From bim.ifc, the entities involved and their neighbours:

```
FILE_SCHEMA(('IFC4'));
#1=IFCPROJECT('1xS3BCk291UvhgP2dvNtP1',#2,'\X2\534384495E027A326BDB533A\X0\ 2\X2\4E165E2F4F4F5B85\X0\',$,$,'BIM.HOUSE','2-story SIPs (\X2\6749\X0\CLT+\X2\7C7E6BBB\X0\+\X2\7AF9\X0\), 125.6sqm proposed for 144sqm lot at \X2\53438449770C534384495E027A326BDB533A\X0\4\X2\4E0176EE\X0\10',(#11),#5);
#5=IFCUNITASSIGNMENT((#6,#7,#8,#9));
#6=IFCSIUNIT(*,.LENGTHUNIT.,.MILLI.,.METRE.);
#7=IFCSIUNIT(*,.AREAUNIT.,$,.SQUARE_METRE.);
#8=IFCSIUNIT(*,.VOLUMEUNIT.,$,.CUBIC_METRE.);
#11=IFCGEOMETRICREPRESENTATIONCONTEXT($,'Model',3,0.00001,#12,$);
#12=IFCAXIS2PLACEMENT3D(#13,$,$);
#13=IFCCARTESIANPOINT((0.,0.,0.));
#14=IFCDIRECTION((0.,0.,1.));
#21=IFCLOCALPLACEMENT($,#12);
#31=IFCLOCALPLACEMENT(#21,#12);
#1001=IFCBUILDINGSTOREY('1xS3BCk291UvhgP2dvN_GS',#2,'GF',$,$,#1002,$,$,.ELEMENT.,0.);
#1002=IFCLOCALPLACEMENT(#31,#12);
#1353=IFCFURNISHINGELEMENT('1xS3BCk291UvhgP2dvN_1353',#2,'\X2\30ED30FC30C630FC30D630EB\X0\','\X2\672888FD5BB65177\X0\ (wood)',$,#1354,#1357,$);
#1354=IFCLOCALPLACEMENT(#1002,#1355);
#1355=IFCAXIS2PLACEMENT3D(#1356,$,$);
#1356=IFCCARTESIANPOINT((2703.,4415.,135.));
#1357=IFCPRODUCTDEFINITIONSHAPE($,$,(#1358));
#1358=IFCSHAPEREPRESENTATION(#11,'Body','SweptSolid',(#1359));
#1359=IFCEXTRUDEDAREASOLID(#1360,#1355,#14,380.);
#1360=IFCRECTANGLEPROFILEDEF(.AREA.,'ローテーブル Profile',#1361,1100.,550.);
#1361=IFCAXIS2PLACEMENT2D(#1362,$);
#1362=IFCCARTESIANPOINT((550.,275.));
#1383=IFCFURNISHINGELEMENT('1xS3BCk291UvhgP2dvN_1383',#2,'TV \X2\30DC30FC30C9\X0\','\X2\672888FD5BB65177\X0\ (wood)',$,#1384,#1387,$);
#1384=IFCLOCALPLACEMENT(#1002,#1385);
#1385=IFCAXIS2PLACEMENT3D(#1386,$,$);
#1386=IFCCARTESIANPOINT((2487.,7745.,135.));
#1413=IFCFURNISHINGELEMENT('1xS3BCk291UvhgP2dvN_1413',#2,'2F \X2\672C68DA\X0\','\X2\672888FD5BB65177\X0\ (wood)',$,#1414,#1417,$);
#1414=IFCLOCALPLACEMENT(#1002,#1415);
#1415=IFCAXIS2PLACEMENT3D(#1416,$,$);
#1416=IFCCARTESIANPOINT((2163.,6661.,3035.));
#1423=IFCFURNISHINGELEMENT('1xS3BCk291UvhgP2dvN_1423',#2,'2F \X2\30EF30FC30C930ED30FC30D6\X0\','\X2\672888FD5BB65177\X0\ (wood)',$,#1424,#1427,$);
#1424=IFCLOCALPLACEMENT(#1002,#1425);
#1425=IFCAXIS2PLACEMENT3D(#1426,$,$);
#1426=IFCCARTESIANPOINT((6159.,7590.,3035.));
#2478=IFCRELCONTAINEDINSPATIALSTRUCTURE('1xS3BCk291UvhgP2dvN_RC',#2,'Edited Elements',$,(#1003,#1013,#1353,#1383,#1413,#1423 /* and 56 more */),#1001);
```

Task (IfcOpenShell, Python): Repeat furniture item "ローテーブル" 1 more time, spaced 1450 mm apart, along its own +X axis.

```python
import ifcopenshell
import ifcopenshell.api.geometry
import ifcopenshell.api.root
import ifcopenshell.util.element
import ifcopenshell.util.placement

model = ifcopenshell.open("bim.ifc")


def reuse_history(source, copy):
    """copy_class also copies each property set's owner history, people and application; keep the originals."""
    for rel in copy.IsDefinedBy:
        if rel.is_a("IfcRelDefinesByProperties") and (history := rel.RelatingPropertyDefinition.OwnerHistory):
            rel.RelatingPropertyDefinition.OwnerHistory = source.OwnerHistory
            ifcopenshell.util.element.remove_deep2(model, history)


source = model.by_guid("1xS3BCk291UvhgP2dvN_1353")
base = ifcopenshell.util.placement.get_local_placement(source.ObjectPlacement)
step = base[:3, 0] * 1450.0

for i in range(1, 2):
    copy = ifcopenshell.api.root.copy_class(model, product=source)
    copy.Representation = ifcopenshell.util.element.copy_deep(
        model, source.Representation, exclude=["IfcGeometricRepresentationContext", "IfcRepresentationMap"]
    )
    reuse_history(source, copy)
    matrix = base.copy()
    matrix[:3, 3] += i * step
    print("added at", matrix[:3, 3].round(3) + 0.0)
    ifcopenshell.api.geometry.edit_object_placement(model, product=copy, matrix=matrix, is_si=False)

model.write("bim_rev.ifc")
```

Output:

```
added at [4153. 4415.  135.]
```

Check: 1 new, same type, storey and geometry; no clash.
